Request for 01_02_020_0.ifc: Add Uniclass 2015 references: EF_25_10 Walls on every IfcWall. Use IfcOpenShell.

First a look at what the model holds.

```python
import ifcopenshell

model = ifcopenshell.open("01_02_020_0.ifc")
print(model.schema)
print("classifications:", [c.Name for c in model.by_type("IfcClassification")])
for ifc_class in ("IfcDoor", "IfcRoof", "IfcStair", "IfcWall", "IfcWindow"):
    print(ifc_class, len(model.by_type(ifc_class)))
```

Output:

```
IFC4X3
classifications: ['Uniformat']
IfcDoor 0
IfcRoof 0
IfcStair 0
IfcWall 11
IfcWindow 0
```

```python
import ifcopenshell
import ifcopenshell.api.classification

model = ifcopenshell.open("01_02_020_0.ifc")

system = ifcopenshell.api.classification.add_classification(model, classification="Uniclass 2015")

codes = {
    "IfcWall": ("EF_25_10", "Walls"),
}
for ifc_class, (code, name) in codes.items():
    products = model.by_type(ifc_class)
    ifcopenshell.api.classification.add_reference(
        model, products=products, classification=system, identification=code, name=name
    )
    print(code, len(products))

model.write("01_02_020_0_updated.ifc")
```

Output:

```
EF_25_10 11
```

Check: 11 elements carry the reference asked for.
